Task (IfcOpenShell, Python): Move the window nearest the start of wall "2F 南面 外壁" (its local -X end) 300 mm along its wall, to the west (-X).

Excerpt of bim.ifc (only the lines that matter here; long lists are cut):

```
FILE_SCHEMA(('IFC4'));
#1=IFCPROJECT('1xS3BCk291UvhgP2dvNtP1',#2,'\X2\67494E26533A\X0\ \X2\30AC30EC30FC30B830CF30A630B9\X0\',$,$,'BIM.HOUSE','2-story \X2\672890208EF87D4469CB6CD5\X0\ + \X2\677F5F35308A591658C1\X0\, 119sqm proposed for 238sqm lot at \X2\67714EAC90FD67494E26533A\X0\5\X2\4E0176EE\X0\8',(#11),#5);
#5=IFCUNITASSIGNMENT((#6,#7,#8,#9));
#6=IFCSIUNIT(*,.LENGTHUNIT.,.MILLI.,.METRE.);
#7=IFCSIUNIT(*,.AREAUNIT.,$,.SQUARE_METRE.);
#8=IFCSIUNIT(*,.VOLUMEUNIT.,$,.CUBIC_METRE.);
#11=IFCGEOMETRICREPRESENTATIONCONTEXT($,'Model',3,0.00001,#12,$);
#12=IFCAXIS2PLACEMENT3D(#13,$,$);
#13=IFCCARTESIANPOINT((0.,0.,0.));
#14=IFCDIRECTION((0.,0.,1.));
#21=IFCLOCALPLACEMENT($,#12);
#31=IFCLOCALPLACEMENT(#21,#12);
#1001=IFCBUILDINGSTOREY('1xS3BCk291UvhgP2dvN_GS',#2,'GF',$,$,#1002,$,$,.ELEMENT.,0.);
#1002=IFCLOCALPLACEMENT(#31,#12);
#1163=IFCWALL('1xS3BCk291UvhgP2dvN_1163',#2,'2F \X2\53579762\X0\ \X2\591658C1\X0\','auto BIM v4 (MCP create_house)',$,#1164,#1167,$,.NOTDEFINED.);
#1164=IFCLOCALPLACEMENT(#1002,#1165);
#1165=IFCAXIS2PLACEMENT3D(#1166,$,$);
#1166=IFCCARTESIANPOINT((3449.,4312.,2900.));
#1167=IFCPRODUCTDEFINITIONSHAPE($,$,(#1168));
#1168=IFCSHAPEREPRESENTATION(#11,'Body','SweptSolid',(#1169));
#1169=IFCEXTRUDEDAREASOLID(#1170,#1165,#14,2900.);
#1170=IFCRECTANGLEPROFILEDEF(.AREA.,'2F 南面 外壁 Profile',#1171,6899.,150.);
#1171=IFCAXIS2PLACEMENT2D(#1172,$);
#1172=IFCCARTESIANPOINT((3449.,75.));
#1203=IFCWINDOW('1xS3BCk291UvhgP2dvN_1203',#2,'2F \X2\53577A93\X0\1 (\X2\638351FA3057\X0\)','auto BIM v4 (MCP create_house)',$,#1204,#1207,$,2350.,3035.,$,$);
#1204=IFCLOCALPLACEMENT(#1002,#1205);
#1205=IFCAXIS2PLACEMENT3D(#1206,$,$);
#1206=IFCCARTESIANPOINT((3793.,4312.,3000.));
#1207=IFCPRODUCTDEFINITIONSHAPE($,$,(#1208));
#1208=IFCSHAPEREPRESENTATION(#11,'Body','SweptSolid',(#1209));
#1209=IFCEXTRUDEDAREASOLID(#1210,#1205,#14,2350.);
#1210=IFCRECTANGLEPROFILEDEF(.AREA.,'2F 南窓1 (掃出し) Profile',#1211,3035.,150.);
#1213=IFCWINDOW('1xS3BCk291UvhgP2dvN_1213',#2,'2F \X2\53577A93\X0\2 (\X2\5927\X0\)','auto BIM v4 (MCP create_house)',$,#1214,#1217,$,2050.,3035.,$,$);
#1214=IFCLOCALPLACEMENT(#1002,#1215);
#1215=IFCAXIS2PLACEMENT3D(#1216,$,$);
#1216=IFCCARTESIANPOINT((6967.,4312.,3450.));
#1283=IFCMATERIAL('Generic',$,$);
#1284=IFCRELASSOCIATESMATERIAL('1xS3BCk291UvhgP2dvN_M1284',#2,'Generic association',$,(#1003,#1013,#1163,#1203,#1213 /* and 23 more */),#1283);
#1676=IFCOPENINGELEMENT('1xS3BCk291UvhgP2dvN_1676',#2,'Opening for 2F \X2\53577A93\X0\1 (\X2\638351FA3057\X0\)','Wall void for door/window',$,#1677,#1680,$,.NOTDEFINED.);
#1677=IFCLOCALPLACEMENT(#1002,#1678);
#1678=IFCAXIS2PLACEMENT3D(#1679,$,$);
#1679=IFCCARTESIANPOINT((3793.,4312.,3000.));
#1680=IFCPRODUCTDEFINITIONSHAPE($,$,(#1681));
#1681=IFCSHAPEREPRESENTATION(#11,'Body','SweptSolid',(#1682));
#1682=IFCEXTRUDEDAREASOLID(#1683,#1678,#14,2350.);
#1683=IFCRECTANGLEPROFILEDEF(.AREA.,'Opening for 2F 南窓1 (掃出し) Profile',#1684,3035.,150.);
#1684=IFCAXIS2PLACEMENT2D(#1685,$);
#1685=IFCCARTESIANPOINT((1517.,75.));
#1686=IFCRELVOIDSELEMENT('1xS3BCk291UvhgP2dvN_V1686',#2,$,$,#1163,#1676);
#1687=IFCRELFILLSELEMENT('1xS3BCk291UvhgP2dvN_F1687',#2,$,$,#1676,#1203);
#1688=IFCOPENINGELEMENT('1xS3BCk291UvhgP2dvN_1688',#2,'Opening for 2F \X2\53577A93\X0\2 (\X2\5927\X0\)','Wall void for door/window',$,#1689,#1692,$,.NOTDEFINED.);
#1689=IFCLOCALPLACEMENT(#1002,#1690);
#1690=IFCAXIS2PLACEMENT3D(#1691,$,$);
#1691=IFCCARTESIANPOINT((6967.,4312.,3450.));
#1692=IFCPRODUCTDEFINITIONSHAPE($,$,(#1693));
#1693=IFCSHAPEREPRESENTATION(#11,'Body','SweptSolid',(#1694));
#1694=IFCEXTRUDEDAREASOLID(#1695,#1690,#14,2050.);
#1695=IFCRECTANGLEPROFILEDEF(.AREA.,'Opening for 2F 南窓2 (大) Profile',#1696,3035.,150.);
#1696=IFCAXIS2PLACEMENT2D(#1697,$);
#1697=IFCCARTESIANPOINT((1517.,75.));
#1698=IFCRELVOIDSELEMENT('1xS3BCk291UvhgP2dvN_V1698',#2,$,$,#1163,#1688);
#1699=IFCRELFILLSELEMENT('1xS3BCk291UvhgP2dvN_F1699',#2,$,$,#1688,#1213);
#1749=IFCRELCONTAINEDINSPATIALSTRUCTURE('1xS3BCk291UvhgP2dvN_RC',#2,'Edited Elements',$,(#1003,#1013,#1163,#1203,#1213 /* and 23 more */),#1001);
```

```python
import ifcopenshell
import ifcopenshell.api.geometry
import ifcopenshell.util.placement
import ifcopenshell.util.unit

model = ifcopenshell.open("bim.ifc")
unit_scale = ifcopenshell.util.unit.calculate_unit_scale(model)

window = model.by_id(1203)
opening = window.FillsVoids[0].RelatingOpeningElement
wall = opening.VoidsElements[0].RelatingBuildingElement

wall_matrix = ifcopenshell.util.placement.get_local_placement(wall.ObjectPlacement)
shift = wall_matrix[:3, 0] * -0.3 / unit_scale
before = ifcopenshell.util.placement.get_local_placement(window.ObjectPlacement)[:3, 3].copy()

# The window is not placed relative to its opening, so move both.
for product in (opening, window):
    matrix = ifcopenshell.util.placement.get_local_placement(product.ObjectPlacement)
    matrix[:3, 3] += shift
    ifcopenshell.api.geometry.edit_object_placement(model, product=product, matrix=matrix, is_si=False)

after = ifcopenshell.util.placement.get_local_placement(window.ObjectPlacement)[:3, 3]
print("window moved by", (after - before).round(3) + 0.0)

model.write("bim_rev.ifc")
```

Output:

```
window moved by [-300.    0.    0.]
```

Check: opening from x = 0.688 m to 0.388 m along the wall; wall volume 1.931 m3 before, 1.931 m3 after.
